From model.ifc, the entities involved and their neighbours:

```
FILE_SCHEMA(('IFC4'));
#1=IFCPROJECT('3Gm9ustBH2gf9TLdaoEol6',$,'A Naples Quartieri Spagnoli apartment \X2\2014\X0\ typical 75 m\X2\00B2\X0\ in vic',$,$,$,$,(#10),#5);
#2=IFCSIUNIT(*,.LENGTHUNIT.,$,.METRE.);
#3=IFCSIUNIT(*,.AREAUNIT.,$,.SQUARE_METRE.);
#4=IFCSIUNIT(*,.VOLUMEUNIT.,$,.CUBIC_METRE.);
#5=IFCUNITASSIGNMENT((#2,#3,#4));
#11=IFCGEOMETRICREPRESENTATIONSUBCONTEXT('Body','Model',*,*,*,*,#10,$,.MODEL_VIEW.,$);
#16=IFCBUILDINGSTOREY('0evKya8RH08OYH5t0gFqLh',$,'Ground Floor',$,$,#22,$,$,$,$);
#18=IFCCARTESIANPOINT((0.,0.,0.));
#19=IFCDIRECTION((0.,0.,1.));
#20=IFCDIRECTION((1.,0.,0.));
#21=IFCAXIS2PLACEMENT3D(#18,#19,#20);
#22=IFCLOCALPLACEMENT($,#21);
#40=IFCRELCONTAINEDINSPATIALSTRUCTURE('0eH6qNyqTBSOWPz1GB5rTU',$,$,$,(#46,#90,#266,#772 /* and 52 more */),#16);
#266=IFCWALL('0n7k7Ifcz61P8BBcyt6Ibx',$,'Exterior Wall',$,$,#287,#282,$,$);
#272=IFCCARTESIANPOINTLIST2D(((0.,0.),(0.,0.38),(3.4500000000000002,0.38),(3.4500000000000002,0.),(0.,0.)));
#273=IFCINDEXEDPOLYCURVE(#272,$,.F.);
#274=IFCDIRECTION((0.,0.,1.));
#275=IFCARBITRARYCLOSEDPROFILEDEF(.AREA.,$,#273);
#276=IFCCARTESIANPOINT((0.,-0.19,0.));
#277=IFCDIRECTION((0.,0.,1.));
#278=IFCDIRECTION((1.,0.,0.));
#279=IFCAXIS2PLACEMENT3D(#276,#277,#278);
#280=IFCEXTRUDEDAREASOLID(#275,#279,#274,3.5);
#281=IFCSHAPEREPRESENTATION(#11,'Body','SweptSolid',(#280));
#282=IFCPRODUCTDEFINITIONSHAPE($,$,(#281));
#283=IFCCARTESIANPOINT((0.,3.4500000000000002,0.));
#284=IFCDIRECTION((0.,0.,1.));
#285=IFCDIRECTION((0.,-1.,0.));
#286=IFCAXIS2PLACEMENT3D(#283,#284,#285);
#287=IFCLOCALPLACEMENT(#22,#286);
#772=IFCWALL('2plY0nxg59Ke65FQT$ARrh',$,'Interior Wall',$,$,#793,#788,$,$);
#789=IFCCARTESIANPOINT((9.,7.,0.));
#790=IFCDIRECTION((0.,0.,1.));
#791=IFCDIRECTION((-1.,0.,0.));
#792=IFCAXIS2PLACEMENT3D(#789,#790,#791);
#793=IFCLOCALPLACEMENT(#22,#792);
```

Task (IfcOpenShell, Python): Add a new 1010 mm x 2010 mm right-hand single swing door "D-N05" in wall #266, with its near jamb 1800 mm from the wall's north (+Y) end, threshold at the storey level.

```python
import numpy as np
import ifcopenshell
import ifcopenshell.api.feature
import ifcopenshell.api.geometry
import ifcopenshell.api.root
import ifcopenshell.api.spatial
import ifcopenshell.geom
import ifcopenshell.util.element
import ifcopenshell.util.placement
import ifcopenshell.util.representation
import ifcopenshell.util.shape
import ifcopenshell.util.unit

model = ifcopenshell.open("model.ifc")
unit_scale = ifcopenshell.util.unit.calculate_unit_scale(model)
settings = ifcopenshell.geom.settings()


def volume(element):
    """Net volume in cubic metres, openings subtracted."""
    shape = ifcopenshell.geom.create_shape(settings, element)
    return ifcopenshell.util.shape.get_volume(shape.geometry)


wall = model.by_guid("0n7k7Ifcz61P8BBcyt6Ibx")
storey = ifcopenshell.util.element.get_container(wall, ifc_class="IfcBuildingStorey")
context = ifcopenshell.util.representation.get_context(model, "Model", "Body", "MODEL_VIEW")
before = volume(wall)

width, height, from_end, sill = 1.01, 2.01, 1.8, 0.0  # metres

# The wall runs along its own X axis, and the end named is its -X end.
wall_shape = ifcopenshell.geom.create_shape(settings, wall)
x, y, z = ifcopenshell.util.shape.get_vertices(wall_shape.geometry).T
start = x.min() + from_end
face, thickness = float(y.min()), float(y.max() - y.min())
wall_matrix = ifcopenshell.util.placement.get_local_placement(wall.ObjectPlacement)
level = ifcopenshell.util.placement.get_local_placement(storey.ObjectPlacement)[2, 3]


def in_wall(x, y):
    """Placement at x, y metres in the wall's axes, at sill height."""
    matrix = wall_matrix.copy()
    matrix[:, 3] = wall_matrix @ np.array([x / unit_scale, y / unit_scale, 0.0, 1.0])
    matrix[2, 3] = level + sill / unit_scale
    return matrix


# Opening: a box that overshoots both wall faces by 50 mm.
opening = ifcopenshell.api.root.create_entity(model, ifc_class="IfcOpeningElement", predefined_type="OPENING")
box = ifcopenshell.api.geometry.add_wall_representation(
    model, context=context, length=width, height=height, thickness=thickness + 0.1
)
ifcopenshell.api.geometry.assign_representation(model, product=opening, representation=box)
ifcopenshell.api.geometry.edit_object_placement(model, product=opening, matrix=in_wall(start, face - 0.05), is_si=False)
ifcopenshell.api.feature.add_feature(model, feature=opening, element=wall)

door = ifcopenshell.api.root.create_entity(model, ifc_class="IfcDoor", name="D-N05", predefined_type="DOOR")
door.OverallWidth, door.OverallHeight = width / unit_scale, height / unit_scale
door.OperationType = "SINGLE_SWING_RIGHT"
body = ifcopenshell.api.geometry.add_door_representation(
    model,
    context=context,
    overall_width=door.OverallWidth,
    overall_height=door.OverallHeight,
    operation_type="SINGLE_SWING_RIGHT",
    lining_properties={"LiningDepth": thickness / unit_scale, "ThresholdDepth": thickness / unit_scale},
)
ifcopenshell.api.geometry.assign_representation(model, product=door, representation=body)
ifcopenshell.api.spatial.assign_container(model, products=[door], relating_structure=storey)
ifcopenshell.api.feature.add_filling(model, opening=opening, element=door)

# The lining spans the wall, so the door starts at the wall face.
ifcopenshell.api.geometry.edit_object_placement(model, product=door, matrix=in_wall(start, face), is_si=False)

after = volume(wall)

print(f"wall volume {before:.3f} -> {after:.3f} m3")

model.write("model_v2.ifc")
```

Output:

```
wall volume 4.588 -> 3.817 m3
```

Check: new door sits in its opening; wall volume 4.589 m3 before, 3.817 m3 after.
